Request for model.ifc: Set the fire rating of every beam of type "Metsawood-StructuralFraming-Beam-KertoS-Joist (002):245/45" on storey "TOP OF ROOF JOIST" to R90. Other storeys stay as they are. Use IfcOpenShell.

First a look at what the model holds.

```python
import ifcopenshell
import ifcopenshell.util.element

model = ifcopenshell.open("model.ifc")
print(model.schema)
storey = next(s for s in model.by_type("IfcBuildingStorey") if s.Name == "TOP OF ROOF JOIST")
beams = [e for e in ifcopenshell.util.element.get_decomposition(storey) if e.is_a("IfcBeam")]
seen = {}
for e in beams:
    element_type = ifcopenshell.util.element.get_type(e)
    key = (element_type.Name if element_type != e and element_type else None, ifcopenshell.util.element.get_pset(e, "Pset_BeamCommon", "FireRating"))
    seen[key] = seen.get(key, 0) + 1
for (name, value), count in sorted(seen.items(), key=str):
    print(count, "x", name, "|", value)
```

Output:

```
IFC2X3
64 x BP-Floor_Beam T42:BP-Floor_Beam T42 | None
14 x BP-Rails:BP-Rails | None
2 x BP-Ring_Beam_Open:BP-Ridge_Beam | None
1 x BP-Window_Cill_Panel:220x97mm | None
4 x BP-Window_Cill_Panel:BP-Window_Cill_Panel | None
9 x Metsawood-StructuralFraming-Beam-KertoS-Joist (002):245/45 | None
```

```python
import ifcopenshell
import ifcopenshell.api.pset
import ifcopenshell.util.element

model = ifcopenshell.open("model.ifc")

storey = next(s for s in model.by_type("IfcBuildingStorey") if s.Name == "TOP OF ROOF JOIST")
beams = [e for e in ifcopenshell.util.element.get_decomposition(storey) if e.is_a("IfcBeam")]

count = 0
for e in beams:
    element_type = ifcopenshell.util.element.get_type(e)
    if element_type in (None, e) or element_type.Name != "Metsawood-StructuralFraming-Beam-KertoS-Joist (002):245/45":
        continue
    # add_pset returns the element's existing set when there is one.
    pset = ifcopenshell.api.pset.add_pset(model, product=e, name="Pset_BeamCommon")
    ifcopenshell.api.pset.edit_pset(model, pset=pset, properties={"FireRating": "R90"})
    count += 1

print(count, "beams updated")

model.write("model_v2.ifc")
```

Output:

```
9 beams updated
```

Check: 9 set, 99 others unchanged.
